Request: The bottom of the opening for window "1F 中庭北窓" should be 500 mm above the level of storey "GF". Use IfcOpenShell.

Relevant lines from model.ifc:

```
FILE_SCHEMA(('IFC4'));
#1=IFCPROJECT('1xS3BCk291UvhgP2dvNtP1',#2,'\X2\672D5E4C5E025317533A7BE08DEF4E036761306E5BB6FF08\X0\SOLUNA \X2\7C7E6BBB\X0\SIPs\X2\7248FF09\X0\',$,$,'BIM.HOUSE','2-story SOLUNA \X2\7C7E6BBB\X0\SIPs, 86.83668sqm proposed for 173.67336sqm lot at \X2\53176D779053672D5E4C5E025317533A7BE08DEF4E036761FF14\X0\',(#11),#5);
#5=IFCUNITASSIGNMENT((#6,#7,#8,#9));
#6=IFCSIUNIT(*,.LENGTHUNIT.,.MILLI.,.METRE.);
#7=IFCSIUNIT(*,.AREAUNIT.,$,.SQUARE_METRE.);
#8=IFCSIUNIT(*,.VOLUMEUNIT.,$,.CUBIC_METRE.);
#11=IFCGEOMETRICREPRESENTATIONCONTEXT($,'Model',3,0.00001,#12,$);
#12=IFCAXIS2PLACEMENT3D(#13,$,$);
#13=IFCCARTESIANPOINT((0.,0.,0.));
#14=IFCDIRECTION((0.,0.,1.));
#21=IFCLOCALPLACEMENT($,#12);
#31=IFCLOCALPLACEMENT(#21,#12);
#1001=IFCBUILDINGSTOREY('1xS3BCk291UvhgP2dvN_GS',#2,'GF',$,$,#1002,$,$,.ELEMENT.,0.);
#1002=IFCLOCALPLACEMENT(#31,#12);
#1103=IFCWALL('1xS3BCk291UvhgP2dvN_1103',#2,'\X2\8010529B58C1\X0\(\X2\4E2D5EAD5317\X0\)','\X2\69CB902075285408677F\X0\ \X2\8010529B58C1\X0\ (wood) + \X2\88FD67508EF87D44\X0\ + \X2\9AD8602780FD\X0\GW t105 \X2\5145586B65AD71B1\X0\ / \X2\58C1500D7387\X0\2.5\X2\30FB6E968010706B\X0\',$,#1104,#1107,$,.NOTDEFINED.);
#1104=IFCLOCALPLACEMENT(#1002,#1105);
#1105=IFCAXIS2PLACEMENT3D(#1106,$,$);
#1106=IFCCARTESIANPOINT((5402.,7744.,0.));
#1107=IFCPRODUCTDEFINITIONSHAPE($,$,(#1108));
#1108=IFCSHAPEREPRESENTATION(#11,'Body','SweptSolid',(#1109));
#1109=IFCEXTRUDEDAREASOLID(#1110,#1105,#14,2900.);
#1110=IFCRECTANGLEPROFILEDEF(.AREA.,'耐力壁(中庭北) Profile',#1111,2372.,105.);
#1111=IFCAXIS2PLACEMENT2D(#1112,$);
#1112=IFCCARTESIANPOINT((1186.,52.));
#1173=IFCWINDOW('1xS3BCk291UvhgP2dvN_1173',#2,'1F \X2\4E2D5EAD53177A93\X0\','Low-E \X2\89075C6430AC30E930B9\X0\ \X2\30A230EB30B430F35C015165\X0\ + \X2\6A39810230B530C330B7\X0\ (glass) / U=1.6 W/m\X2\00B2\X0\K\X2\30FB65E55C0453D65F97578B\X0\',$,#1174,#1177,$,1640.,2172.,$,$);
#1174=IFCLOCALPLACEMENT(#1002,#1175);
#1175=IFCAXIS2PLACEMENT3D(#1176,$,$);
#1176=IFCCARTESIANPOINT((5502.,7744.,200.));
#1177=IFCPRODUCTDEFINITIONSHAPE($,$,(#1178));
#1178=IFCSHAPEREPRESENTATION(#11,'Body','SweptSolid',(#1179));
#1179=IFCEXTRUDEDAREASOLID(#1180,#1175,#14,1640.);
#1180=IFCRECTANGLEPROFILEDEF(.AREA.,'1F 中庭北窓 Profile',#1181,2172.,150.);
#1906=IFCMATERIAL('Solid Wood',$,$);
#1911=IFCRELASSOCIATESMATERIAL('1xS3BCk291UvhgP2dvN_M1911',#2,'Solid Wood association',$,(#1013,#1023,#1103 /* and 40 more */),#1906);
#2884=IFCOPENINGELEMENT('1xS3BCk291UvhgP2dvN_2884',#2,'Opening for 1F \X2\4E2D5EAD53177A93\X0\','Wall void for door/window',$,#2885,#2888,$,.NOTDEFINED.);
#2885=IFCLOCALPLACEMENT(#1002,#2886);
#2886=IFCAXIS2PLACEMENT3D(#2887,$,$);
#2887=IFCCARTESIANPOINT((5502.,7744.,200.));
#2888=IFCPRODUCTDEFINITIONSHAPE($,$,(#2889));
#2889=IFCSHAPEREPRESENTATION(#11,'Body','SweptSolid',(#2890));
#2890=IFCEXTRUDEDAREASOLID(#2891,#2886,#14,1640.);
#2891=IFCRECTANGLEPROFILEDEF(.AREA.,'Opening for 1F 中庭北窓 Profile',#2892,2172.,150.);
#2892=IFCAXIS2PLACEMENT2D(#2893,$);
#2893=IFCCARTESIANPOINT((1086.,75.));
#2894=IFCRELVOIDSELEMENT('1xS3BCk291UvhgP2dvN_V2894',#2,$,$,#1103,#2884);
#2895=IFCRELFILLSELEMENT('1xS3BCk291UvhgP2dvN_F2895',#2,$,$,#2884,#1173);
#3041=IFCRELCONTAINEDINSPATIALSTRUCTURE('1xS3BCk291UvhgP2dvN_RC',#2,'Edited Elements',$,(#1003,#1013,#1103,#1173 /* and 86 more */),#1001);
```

```python
import numpy as np
import ifcopenshell
import ifcopenshell.api.geometry
import ifcopenshell.geom
import ifcopenshell.util.element
import ifcopenshell.util.placement
import ifcopenshell.util.shape
import ifcopenshell.util.unit

model = ifcopenshell.open("model.ifc")
unit_scale = ifcopenshell.util.unit.calculate_unit_scale(model)

window = model.by_id(1173)
opening = window.FillsVoids[0].RelatingOpeningElement
storey = ifcopenshell.util.element.get_container(window, ifc_class="IfcBuildingStorey")
level = ifcopenshell.util.placement.get_local_placement(storey.ObjectPlacement)[2, 3]

# The opening's origin need not be at the sill, so measure its lowest point.
shape = ifcopenshell.geom.create_shape(ifcopenshell.geom.settings(), opening)
bottom = ifcopenshell.util.shape.get_shape_bottom_elevation(shape, shape.geometry) / unit_scale
dz = level + 500.0 - bottom

shift = np.array([0.0, 0.0, dz])
# The window is not placed relative to its opening, so move both.
for product in (opening, window):
    matrix = ifcopenshell.util.placement.get_local_placement(product.ObjectPlacement)
    matrix[:3, 3] += shift
    ifcopenshell.api.geometry.edit_object_placement(model, product=product, matrix=matrix, is_si=False)

print(f"moved by {dz * unit_scale:+.3f} m")

model.write("model_rev.ifc")
```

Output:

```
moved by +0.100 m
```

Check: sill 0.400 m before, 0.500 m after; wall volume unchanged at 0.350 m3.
